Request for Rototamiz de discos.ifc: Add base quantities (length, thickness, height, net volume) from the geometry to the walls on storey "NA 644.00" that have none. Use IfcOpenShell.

First a look at what the model holds.

```python
import ifcopenshell
import ifcopenshell.util.element
import ifcopenshell.util.unit

model = ifcopenshell.open("Rototamiz de discos.ifc")
print(model.schema)
for unit_type in ("LENGTHUNIT", "AREAUNIT", "VOLUMEUNIT"):
    print(unit_type, ifcopenshell.util.unit.calculate_unit_scale(model, unit_type))
storey = next(s for s in model.by_type("IfcBuildingStorey") if s.Name == "NA 644.00")
walls = [e for e in ifcopenshell.util.element.get_decomposition(storey) if e.is_a("IfcWall")]
for e in sorted(walls, key=lambda e: e.id()):
    print(e.id(), e.is_a(), e.Name, list(ifcopenshell.util.element.get_psets(e, qtos_only=True)), sep=" | ")
```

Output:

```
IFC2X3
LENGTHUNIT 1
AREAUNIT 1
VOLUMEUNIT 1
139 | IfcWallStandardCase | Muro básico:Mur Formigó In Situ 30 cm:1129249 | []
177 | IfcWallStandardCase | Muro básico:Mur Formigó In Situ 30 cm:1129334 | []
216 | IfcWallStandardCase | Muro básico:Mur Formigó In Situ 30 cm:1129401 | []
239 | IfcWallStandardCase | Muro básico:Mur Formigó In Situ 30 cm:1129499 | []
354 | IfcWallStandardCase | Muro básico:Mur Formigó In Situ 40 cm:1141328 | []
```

```python
import ifcopenshell
import ifcopenshell.api.pset
import ifcopenshell.geom
import ifcopenshell.util.element
import ifcopenshell.util.shape
import ifcopenshell.util.unit

model = ifcopenshell.open("Rototamiz de discos.ifc")
unit_scale = ifcopenshell.util.unit.calculate_unit_scale(model)
volume_scale = ifcopenshell.util.unit.calculate_unit_scale(model, "VOLUMEUNIT")
settings = ifcopenshell.geom.settings()

storey = next(s for s in model.by_type("IfcBuildingStorey") if s.Name == "NA 644.00")
walls = [e for e in ifcopenshell.util.element.get_decomposition(storey) if e.is_a("IfcWall")]

for e in sorted(walls, key=lambda e: e.id()):
    if ifcopenshell.util.element.get_psets(e, qtos_only=True, should_inherit=False):
        continue
    # Geometry comes back in metres, in the element's own axes.
    shape = ifcopenshell.geom.create_shape(settings, e)
    values = {
        "Length": ifcopenshell.util.shape.get_x(shape.geometry) / unit_scale,
        "Width": ifcopenshell.util.shape.get_y(shape.geometry) / unit_scale,
        "Height": ifcopenshell.util.shape.get_z(shape.geometry) / unit_scale,
        "NetVolume": ifcopenshell.util.shape.get_volume(shape.geometry) / volume_scale,
    }
    qto = ifcopenshell.api.pset.add_qto(model, product=e, name="BaseQuantities")
    ifcopenshell.api.pset.edit_qto(model, qto=qto, properties=values)
    print(e.id(), {k: round(v, 3) for k, v in values.items()})

model.write("Rototamiz de discos_rev.ifc")
```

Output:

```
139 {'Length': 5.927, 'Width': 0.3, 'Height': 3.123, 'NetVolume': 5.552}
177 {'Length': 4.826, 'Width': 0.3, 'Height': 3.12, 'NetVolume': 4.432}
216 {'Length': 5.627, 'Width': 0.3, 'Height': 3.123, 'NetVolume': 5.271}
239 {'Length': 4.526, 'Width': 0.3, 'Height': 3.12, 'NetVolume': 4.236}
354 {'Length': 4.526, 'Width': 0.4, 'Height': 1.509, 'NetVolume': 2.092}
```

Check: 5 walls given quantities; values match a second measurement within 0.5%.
